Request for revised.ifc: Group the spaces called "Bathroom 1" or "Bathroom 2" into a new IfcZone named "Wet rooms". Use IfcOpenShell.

First a look at what the model holds.

```python
import ifcopenshell

model = ifcopenshell.open("revised.ifc")
print(model.schema)
seen = {}
for space in model.by_type("IfcSpace"):
    seen[space.LongName] = seen.get(space.LongName, 0) + 1
for name, count in sorted(seen.items(), key=str):
    print(count, "x", name)
print("zones:", [z.Name for z in model.by_type("IfcZone")][:20])
```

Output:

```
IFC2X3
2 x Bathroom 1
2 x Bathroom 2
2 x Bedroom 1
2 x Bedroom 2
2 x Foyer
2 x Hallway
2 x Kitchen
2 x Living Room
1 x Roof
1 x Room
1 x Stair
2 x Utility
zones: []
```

```python
import ifcopenshell
import ifcopenshell.api.group
import ifcopenshell.api.root

model = ifcopenshell.open("revised.ifc")

names = {"Bathroom 1", "Bathroom 2"}
spaces = [s for s in model.by_type("IfcSpace") if s.LongName in names]

zone = ifcopenshell.api.root.create_entity(model, ifc_class="IfcZone", name="Wet rooms")
ifcopenshell.api.group.assign_group(model, products=spaces, group=zone)
print(len(spaces), "spaces in", zone.Name)

model.write("revised_updated.ifc")
```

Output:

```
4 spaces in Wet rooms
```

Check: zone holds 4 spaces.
